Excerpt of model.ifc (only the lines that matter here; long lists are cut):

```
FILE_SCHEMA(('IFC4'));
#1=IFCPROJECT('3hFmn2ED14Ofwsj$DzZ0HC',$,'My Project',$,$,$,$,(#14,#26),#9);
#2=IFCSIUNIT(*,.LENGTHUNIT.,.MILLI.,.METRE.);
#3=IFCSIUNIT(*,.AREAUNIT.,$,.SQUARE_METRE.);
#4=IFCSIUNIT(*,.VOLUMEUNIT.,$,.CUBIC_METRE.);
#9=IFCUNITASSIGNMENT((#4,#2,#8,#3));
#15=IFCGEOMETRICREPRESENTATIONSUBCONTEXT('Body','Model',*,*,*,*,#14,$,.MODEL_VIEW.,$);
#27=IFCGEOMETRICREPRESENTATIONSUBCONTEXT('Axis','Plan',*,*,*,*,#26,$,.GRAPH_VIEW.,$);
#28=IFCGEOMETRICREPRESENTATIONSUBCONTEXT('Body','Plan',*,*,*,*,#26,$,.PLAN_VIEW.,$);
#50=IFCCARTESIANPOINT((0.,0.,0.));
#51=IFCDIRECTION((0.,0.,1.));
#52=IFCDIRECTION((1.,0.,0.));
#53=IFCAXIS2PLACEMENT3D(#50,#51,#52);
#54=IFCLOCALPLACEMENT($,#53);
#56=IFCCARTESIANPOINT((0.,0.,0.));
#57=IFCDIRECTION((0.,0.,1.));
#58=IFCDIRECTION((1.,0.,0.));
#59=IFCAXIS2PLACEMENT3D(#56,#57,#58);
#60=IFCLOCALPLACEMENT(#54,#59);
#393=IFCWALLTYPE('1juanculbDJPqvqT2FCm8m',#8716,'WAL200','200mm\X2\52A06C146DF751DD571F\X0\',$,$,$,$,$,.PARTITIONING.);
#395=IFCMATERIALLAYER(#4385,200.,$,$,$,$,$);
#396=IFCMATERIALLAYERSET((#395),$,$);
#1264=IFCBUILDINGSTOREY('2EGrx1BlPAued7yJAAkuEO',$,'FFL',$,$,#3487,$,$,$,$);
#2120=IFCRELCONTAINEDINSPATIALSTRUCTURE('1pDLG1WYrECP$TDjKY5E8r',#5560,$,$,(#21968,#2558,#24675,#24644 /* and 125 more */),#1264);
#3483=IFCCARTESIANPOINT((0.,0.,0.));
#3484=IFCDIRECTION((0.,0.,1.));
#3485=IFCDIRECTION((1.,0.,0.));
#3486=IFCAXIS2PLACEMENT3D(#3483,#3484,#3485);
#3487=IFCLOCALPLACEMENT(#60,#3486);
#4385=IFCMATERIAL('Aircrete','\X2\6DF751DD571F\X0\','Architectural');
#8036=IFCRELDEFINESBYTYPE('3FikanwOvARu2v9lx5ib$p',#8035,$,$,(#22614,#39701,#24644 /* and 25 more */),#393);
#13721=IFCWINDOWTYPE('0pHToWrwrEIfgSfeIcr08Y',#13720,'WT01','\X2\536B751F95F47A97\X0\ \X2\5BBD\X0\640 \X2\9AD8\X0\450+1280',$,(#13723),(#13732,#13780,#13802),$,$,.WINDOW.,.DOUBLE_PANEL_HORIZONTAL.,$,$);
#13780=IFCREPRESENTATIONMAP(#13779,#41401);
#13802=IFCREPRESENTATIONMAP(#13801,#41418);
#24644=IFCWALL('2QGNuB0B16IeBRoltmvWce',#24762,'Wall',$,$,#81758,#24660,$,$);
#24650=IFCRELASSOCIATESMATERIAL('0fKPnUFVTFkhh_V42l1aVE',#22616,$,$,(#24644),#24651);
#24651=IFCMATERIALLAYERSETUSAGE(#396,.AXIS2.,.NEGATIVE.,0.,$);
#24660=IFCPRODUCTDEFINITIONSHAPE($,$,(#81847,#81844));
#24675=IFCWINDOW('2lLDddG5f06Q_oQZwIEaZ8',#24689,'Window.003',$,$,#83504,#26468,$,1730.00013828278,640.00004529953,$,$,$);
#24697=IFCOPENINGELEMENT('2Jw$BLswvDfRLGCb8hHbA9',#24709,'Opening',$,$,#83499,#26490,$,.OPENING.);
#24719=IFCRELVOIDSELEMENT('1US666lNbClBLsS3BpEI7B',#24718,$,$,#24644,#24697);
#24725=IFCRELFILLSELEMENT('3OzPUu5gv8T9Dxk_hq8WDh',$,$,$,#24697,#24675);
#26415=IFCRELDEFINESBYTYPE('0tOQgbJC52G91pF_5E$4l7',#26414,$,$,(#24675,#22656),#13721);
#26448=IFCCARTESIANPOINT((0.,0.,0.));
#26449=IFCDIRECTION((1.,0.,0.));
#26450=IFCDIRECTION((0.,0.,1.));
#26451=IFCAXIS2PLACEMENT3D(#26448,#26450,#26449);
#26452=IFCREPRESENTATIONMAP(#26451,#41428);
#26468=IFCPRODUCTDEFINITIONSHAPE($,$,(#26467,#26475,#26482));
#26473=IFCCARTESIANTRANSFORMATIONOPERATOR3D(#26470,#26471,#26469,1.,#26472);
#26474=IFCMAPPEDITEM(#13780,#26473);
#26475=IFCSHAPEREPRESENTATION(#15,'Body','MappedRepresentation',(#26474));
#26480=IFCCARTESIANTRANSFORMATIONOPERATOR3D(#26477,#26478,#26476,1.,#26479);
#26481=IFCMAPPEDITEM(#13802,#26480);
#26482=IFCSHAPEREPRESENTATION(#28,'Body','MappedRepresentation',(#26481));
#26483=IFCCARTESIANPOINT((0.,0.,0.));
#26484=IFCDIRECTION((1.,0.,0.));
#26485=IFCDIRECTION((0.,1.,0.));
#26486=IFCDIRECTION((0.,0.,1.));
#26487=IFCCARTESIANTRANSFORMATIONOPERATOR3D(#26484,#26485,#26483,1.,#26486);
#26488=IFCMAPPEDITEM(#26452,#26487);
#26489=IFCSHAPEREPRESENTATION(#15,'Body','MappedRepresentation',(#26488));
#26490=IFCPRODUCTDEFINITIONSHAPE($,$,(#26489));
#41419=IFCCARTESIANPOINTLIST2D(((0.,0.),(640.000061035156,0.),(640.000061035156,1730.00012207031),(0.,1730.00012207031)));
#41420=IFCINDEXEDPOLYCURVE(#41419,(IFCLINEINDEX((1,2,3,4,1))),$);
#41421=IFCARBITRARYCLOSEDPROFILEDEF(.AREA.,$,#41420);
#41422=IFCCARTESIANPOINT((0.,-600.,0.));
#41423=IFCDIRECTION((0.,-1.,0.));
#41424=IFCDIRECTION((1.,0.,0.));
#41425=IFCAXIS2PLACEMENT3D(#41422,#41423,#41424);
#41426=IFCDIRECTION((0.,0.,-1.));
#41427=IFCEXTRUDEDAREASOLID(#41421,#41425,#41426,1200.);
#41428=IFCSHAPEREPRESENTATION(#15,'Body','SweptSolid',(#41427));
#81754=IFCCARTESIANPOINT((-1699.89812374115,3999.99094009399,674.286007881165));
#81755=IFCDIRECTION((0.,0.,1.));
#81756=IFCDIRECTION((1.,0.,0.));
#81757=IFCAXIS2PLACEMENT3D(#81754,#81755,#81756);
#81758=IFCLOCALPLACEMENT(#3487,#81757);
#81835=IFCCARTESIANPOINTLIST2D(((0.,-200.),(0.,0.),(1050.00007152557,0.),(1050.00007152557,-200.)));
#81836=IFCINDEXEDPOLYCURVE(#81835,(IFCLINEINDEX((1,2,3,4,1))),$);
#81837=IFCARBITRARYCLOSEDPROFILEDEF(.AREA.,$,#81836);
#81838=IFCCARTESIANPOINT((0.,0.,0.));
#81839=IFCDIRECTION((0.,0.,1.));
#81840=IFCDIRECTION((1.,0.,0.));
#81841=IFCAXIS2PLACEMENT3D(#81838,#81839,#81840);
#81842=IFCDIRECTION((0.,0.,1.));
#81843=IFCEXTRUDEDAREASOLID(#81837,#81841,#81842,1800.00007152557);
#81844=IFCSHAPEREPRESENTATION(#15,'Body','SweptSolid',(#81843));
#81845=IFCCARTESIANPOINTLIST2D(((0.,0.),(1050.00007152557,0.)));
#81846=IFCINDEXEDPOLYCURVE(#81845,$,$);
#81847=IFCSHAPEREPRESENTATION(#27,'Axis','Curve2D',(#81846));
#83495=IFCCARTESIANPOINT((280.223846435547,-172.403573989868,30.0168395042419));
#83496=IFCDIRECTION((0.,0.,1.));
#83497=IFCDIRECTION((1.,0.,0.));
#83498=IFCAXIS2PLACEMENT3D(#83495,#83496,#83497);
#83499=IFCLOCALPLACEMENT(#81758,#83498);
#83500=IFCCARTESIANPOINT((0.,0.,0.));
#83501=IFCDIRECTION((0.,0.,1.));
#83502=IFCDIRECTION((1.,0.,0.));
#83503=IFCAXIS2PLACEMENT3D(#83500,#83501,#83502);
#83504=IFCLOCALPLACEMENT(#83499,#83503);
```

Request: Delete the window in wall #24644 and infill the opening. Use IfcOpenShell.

```python
import ifcopenshell
import ifcopenshell.api.feature
import ifcopenshell.api.root
import ifcopenshell.geom
import ifcopenshell.util.shape

model = ifcopenshell.open("model.ifc")
settings = ifcopenshell.geom.settings()


def volume(element):
    """Net volume in cubic metres, openings subtracted."""
    shape = ifcopenshell.geom.create_shape(settings, element)
    return ifcopenshell.util.shape.get_volume(shape.geometry)


window = model.by_guid("2lLDddG5f06Q_oQZwIEaZ8")
opening = window.FillsVoids[0].RelatingOpeningElement
wall = opening.VoidsElements[0].RelatingBuildingElement
before = volume(wall)

ifcopenshell.api.root.remove_product(model, product=window)
ifcopenshell.api.feature.remove_feature(model, feature=opening)

after = volume(wall)

print(f"wall volume {before:.3f} -> {after:.3f} m3")

model.write("model_v2.ifc")
```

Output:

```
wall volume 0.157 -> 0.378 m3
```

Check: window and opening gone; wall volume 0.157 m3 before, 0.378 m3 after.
